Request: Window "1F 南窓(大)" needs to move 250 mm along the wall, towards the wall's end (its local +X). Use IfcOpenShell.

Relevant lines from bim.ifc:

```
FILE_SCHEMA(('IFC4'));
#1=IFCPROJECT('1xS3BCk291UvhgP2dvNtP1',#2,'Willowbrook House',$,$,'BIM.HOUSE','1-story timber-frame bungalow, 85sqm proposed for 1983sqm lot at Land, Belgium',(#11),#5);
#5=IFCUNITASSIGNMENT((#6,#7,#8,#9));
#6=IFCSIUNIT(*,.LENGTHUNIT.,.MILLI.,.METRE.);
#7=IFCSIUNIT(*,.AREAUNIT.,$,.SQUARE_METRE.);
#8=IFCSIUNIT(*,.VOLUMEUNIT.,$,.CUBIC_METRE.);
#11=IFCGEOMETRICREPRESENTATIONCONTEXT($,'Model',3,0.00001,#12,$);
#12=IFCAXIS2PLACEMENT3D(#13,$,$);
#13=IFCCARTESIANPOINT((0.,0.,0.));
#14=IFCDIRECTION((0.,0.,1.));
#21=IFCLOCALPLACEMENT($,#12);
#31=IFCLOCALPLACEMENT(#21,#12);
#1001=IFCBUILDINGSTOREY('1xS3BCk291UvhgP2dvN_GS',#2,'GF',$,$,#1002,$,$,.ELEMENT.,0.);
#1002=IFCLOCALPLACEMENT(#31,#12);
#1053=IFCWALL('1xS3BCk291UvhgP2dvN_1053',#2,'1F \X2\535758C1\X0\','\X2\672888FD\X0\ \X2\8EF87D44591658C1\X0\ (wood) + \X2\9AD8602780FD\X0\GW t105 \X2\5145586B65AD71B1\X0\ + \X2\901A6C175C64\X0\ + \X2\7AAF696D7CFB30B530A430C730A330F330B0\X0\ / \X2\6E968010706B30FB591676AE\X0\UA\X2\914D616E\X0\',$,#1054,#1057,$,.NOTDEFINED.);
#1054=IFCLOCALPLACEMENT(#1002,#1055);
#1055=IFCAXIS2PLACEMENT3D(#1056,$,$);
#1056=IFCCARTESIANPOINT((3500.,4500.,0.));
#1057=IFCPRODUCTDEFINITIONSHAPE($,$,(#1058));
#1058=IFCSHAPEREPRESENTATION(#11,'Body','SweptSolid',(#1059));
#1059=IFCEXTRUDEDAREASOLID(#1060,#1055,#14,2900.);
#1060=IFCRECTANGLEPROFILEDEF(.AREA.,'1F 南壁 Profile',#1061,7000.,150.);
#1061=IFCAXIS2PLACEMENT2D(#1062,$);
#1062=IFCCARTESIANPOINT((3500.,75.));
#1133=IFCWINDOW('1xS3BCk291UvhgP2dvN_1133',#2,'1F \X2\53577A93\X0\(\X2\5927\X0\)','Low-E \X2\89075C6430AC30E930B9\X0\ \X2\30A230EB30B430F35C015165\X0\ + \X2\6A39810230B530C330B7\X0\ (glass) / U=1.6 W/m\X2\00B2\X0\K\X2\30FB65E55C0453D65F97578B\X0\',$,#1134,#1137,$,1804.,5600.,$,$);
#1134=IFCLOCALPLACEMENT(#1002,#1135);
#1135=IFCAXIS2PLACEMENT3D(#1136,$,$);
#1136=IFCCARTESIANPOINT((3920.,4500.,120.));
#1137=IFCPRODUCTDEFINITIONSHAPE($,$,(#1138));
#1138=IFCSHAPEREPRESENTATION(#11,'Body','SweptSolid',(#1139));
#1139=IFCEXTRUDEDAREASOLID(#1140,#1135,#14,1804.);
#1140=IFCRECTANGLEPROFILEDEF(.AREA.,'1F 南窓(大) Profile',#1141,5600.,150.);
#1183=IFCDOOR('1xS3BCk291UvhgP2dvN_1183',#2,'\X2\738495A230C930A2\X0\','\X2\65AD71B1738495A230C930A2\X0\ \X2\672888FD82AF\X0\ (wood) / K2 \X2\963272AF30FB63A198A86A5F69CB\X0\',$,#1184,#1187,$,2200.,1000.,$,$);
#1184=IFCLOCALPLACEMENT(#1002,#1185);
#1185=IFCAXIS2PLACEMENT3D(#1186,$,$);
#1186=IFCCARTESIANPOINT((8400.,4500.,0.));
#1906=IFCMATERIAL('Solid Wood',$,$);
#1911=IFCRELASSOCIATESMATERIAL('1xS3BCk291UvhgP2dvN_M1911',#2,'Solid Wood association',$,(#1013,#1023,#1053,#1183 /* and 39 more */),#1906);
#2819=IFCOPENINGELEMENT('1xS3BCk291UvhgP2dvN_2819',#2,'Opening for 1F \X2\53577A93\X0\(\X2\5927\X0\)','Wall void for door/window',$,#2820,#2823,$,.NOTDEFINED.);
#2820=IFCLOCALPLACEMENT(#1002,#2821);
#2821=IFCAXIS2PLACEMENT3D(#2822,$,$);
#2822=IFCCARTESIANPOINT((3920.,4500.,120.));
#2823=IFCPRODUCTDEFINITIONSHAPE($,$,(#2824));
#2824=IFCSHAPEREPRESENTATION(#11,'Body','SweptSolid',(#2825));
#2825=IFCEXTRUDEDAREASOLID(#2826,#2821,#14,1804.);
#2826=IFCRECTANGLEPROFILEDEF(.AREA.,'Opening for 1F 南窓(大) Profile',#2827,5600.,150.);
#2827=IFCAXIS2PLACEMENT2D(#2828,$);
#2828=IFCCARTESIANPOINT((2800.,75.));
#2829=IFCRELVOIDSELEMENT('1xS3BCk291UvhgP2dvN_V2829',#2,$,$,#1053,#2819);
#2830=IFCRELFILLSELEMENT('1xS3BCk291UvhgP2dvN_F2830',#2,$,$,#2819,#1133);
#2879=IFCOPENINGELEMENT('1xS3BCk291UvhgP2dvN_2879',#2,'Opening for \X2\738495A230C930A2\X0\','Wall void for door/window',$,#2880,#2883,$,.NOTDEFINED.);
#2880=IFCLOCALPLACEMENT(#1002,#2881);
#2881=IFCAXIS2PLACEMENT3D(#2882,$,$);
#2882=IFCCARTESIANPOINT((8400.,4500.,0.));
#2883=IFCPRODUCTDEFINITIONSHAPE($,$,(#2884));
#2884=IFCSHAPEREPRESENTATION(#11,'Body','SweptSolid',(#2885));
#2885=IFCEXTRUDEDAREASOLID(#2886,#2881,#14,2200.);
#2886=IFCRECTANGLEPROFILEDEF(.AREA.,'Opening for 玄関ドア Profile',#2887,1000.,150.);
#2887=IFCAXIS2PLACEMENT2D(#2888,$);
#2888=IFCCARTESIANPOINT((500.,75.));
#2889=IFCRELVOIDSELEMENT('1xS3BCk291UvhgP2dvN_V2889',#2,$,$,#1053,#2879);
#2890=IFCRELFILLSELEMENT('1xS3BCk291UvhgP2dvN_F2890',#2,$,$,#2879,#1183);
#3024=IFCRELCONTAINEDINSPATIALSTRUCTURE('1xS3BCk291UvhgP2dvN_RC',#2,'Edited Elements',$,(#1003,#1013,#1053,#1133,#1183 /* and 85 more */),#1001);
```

```python
import ifcopenshell
import ifcopenshell.api.geometry
import ifcopenshell.util.placement

model = ifcopenshell.open("bim.ifc")

window = model.by_guid("1xS3BCk291UvhgP2dvN_1133")
opening = window.FillsVoids[0].RelatingOpeningElement
wall = opening.VoidsElements[0].RelatingBuildingElement

wall_matrix = ifcopenshell.util.placement.get_local_placement(wall.ObjectPlacement)
shift = wall_matrix[:3, 0] * 250.0
before = ifcopenshell.util.placement.get_local_placement(window.ObjectPlacement)[:3, 3].copy()

# The window is not placed relative to its opening, so move both.
for product in (opening, window):
    matrix = ifcopenshell.util.placement.get_local_placement(product.ObjectPlacement)
    matrix[:3, 3] += shift
    ifcopenshell.api.geometry.edit_object_placement(model, product=product, matrix=matrix, is_si=False)

after = ifcopenshell.util.placement.get_local_placement(window.ObjectPlacement)[:3, 3]
print("window moved by", (after - before).round(3) + 0.0)

model.write("bim_rev.ifc")
```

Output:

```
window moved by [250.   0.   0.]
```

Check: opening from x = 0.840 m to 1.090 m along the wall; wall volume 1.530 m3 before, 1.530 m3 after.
